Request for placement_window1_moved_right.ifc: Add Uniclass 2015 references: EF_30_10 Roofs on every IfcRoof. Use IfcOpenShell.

First a look at what the model holds.

```python
import ifcopenshell

model = ifcopenshell.open("placement_window1_moved_right.ifc")
print(model.schema)
print("classifications:", [c.Name for c in model.by_type("IfcClassification")])
for ifc_class in ("IfcDoor", "IfcRoof", "IfcStair", "IfcWall", "IfcWindow"):
    print(ifc_class, len(model.by_type(ifc_class)))
```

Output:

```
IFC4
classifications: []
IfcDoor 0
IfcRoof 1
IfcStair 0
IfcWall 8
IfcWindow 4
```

```python
import ifcopenshell
import ifcopenshell.api.classification

model = ifcopenshell.open("placement_window1_moved_right.ifc")

system = ifcopenshell.api.classification.add_classification(model, classification="Uniclass 2015")

codes = {
    "IfcRoof": ("EF_30_10", "Roofs"),
}
for ifc_class, (code, name) in codes.items():
    products = model.by_type(ifc_class)
    ifcopenshell.api.classification.add_reference(
        model, products=products, classification=system, identification=code, name=name
    )
    print(code, len(products))

model.write("placement_window1_moved_right_v2.ifc")
```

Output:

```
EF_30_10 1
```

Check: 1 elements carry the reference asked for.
